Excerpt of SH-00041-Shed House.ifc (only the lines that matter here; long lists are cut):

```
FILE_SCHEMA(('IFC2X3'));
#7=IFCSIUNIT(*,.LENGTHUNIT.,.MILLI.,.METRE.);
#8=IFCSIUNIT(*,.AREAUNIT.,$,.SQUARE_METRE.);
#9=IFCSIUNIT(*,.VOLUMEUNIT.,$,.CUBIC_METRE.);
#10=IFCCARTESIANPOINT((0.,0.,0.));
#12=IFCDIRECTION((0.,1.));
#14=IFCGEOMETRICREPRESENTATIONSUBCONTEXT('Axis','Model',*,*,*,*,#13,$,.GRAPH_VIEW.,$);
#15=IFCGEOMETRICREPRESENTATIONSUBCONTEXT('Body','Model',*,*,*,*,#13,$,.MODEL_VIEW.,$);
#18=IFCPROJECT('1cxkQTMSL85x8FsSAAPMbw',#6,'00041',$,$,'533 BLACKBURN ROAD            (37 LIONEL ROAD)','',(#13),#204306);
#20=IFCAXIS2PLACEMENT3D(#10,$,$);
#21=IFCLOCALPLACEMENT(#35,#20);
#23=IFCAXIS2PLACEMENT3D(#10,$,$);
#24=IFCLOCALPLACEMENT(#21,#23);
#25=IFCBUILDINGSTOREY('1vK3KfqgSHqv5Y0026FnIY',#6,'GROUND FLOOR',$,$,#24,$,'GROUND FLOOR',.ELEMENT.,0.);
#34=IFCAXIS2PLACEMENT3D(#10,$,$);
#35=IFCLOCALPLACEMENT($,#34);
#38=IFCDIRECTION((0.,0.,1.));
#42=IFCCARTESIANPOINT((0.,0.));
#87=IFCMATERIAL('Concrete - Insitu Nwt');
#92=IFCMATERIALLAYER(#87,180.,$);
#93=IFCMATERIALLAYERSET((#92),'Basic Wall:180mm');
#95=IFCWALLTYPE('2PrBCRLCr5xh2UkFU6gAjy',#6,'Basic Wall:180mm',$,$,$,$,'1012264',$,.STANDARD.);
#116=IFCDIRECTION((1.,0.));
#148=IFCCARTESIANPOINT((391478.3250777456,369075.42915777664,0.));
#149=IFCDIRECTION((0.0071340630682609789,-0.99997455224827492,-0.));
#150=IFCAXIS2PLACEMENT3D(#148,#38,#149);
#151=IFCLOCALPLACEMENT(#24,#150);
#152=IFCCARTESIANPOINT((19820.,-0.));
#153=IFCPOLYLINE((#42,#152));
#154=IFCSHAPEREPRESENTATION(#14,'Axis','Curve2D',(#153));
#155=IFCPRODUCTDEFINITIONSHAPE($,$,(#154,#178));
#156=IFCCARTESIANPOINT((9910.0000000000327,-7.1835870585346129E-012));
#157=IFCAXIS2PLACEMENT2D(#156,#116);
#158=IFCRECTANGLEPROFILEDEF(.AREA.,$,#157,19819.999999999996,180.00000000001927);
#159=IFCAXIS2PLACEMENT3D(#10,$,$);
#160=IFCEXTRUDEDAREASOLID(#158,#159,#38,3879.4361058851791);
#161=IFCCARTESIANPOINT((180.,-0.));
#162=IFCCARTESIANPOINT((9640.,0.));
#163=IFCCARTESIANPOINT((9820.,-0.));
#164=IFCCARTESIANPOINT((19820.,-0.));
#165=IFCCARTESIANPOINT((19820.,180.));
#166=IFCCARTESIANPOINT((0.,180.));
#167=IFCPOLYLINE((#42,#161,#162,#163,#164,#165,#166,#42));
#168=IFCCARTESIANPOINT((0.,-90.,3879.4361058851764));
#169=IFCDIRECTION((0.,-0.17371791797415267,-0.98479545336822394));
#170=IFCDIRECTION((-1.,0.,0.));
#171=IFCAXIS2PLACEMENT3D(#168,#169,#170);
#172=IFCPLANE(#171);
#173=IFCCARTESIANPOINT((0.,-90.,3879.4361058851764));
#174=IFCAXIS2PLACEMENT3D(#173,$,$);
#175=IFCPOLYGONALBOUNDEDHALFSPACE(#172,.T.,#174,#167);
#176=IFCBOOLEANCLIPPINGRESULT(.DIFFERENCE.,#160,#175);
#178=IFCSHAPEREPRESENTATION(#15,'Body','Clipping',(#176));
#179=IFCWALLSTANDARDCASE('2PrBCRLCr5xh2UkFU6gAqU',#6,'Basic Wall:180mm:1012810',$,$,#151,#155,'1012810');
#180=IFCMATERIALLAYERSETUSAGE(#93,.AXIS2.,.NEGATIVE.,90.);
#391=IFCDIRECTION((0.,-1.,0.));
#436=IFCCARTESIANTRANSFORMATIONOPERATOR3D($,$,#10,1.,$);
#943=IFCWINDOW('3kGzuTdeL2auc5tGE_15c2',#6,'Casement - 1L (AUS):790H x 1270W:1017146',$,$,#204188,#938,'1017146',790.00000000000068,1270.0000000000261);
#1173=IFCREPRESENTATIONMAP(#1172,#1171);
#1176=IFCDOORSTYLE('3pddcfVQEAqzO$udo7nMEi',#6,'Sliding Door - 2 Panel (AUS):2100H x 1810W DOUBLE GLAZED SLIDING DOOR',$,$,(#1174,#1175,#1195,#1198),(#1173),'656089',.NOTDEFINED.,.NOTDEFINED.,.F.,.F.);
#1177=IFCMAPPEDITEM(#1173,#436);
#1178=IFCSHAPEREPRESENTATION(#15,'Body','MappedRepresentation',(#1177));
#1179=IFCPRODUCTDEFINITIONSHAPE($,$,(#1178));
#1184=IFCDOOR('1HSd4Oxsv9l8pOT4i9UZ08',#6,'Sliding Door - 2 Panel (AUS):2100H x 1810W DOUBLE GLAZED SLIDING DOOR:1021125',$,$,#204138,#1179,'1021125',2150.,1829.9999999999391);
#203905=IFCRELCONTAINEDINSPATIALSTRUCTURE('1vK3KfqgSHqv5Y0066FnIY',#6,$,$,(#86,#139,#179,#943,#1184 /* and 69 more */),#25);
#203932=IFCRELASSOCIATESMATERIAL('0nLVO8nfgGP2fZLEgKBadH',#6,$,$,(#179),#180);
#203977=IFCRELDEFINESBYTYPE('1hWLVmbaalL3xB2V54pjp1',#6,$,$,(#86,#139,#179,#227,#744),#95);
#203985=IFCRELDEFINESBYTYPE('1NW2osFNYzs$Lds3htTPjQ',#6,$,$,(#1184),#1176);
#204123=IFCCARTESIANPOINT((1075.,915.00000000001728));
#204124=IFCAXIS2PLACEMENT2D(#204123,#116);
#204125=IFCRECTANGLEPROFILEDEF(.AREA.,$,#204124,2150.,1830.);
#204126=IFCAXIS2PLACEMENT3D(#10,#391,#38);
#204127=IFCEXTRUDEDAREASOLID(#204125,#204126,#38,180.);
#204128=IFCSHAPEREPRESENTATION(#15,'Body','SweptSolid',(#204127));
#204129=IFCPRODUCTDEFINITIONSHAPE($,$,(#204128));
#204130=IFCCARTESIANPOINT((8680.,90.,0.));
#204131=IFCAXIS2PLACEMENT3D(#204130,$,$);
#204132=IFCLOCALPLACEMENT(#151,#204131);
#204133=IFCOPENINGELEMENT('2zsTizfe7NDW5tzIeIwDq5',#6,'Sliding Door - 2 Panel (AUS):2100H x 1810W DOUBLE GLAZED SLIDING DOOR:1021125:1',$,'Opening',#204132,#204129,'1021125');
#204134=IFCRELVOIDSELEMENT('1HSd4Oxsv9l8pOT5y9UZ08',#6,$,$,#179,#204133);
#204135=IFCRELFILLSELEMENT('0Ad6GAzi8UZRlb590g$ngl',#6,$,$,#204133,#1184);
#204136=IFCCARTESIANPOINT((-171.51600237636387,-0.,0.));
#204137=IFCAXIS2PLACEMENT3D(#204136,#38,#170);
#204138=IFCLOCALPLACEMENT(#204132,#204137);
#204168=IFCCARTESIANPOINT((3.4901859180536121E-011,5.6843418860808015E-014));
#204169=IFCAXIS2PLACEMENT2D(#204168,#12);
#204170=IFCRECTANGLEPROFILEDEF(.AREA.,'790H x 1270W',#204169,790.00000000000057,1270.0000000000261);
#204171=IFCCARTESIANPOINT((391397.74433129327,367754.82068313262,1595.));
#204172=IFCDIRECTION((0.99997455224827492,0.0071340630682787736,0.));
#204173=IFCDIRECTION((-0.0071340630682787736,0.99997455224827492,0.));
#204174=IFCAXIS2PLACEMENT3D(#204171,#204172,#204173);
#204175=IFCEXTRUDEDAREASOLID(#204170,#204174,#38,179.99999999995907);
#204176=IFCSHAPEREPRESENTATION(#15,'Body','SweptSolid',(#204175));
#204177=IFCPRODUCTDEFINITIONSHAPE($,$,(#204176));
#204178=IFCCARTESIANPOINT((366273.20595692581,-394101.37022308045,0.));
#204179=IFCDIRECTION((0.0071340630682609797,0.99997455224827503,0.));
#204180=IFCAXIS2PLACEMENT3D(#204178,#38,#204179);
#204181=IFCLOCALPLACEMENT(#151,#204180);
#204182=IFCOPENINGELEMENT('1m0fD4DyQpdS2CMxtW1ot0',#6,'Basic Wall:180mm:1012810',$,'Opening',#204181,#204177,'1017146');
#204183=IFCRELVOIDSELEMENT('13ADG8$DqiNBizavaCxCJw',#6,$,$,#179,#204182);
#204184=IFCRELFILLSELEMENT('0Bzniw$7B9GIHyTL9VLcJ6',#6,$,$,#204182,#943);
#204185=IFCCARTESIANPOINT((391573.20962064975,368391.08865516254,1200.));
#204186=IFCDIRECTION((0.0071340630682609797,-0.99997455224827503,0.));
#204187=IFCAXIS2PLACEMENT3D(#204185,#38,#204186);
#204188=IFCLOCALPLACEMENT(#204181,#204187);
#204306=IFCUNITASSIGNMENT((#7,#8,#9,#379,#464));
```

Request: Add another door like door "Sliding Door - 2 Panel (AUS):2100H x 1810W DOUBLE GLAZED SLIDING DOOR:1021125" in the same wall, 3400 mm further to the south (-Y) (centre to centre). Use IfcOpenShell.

```python
import ifcopenshell
import ifcopenshell.api.feature
import ifcopenshell.api.geometry
import ifcopenshell.api.root
import ifcopenshell.geom
import ifcopenshell.util.element
import ifcopenshell.util.placement
import ifcopenshell.util.shape
import ifcopenshell.util.unit

model = ifcopenshell.open("SH-00041-Shed House.ifc")
unit_scale = ifcopenshell.util.unit.calculate_unit_scale(model)
settings = ifcopenshell.geom.settings()


def volume(element):
    """Net volume in cubic metres, openings subtracted."""
    shape = ifcopenshell.geom.create_shape(settings, element)
    return ifcopenshell.util.shape.get_volume(shape.geometry)


def reuse_history(source, copy):
    """copy_class also copies each property set's owner history, people and application; keep the originals."""
    for rel in copy.IsDefinedBy:
        if rel.is_a("IfcRelDefinesByProperties") and (history := rel.RelatingPropertyDefinition.OwnerHistory):
            rel.RelatingPropertyDefinition.OwnerHistory = source.OwnerHistory
            ifcopenshell.util.element.remove_deep2(model, history)


door = model.by_id(1184)
opening = door.FillsVoids[0].RelatingOpeningElement
wall = opening.VoidsElements[0].RelatingBuildingElement
before = volume(wall)
shift = ifcopenshell.util.placement.get_local_placement(wall.ObjectPlacement)[:3, 0] * 3.4 / unit_scale

# copy_class copies the void relationship, type, container and properties, but no geometry.
new_opening = ifcopenshell.api.root.copy_class(model, product=opening)
new_opening.Representation = ifcopenshell.util.element.copy_deep(
    model, opening.Representation, exclude=["IfcGeometricRepresentationContext", "IfcRepresentationMap"]
)
new_opening.Name = "Sliding Door - 2 Panel (AUS):2100H x 1810W DOUBLE GLAZED SLIDING DOOR"
new_opening.Tag = None
new_door = ifcopenshell.api.root.copy_class(model, product=door)
new_door.Representation = ifcopenshell.util.element.copy_deep(
    model, door.Representation, exclude=["IfcGeometricRepresentationContext", "IfcRepresentationMap"]
)
new_door.Name = "Sliding Door - 2 Panel (AUS):2100H x 1810W DOUBLE GLAZED SLIDING DOOR"
new_door.Tag = None
reuse_history(door, new_door)
fills = ifcopenshell.api.feature.add_filling(model, opening=new_opening, element=new_door)
fills.OwnerHistory = new_door.OwnerHistory  # required in IFC2X3

for old, new in ((opening, new_opening), (door, new_door)):
    matrix = ifcopenshell.util.placement.get_local_placement(old.ObjectPlacement)
    matrix[:3, 3] += shift
    ifcopenshell.api.geometry.edit_object_placement(model, product=new, matrix=matrix, is_si=False)

after = volume(wall)

print(f"wall volume {before:.3f} -> {after:.3f} m3")

model.write("SH-00041-Shed House_v2.ifc")
```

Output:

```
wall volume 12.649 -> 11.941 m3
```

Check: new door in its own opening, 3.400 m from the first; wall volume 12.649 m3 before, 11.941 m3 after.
